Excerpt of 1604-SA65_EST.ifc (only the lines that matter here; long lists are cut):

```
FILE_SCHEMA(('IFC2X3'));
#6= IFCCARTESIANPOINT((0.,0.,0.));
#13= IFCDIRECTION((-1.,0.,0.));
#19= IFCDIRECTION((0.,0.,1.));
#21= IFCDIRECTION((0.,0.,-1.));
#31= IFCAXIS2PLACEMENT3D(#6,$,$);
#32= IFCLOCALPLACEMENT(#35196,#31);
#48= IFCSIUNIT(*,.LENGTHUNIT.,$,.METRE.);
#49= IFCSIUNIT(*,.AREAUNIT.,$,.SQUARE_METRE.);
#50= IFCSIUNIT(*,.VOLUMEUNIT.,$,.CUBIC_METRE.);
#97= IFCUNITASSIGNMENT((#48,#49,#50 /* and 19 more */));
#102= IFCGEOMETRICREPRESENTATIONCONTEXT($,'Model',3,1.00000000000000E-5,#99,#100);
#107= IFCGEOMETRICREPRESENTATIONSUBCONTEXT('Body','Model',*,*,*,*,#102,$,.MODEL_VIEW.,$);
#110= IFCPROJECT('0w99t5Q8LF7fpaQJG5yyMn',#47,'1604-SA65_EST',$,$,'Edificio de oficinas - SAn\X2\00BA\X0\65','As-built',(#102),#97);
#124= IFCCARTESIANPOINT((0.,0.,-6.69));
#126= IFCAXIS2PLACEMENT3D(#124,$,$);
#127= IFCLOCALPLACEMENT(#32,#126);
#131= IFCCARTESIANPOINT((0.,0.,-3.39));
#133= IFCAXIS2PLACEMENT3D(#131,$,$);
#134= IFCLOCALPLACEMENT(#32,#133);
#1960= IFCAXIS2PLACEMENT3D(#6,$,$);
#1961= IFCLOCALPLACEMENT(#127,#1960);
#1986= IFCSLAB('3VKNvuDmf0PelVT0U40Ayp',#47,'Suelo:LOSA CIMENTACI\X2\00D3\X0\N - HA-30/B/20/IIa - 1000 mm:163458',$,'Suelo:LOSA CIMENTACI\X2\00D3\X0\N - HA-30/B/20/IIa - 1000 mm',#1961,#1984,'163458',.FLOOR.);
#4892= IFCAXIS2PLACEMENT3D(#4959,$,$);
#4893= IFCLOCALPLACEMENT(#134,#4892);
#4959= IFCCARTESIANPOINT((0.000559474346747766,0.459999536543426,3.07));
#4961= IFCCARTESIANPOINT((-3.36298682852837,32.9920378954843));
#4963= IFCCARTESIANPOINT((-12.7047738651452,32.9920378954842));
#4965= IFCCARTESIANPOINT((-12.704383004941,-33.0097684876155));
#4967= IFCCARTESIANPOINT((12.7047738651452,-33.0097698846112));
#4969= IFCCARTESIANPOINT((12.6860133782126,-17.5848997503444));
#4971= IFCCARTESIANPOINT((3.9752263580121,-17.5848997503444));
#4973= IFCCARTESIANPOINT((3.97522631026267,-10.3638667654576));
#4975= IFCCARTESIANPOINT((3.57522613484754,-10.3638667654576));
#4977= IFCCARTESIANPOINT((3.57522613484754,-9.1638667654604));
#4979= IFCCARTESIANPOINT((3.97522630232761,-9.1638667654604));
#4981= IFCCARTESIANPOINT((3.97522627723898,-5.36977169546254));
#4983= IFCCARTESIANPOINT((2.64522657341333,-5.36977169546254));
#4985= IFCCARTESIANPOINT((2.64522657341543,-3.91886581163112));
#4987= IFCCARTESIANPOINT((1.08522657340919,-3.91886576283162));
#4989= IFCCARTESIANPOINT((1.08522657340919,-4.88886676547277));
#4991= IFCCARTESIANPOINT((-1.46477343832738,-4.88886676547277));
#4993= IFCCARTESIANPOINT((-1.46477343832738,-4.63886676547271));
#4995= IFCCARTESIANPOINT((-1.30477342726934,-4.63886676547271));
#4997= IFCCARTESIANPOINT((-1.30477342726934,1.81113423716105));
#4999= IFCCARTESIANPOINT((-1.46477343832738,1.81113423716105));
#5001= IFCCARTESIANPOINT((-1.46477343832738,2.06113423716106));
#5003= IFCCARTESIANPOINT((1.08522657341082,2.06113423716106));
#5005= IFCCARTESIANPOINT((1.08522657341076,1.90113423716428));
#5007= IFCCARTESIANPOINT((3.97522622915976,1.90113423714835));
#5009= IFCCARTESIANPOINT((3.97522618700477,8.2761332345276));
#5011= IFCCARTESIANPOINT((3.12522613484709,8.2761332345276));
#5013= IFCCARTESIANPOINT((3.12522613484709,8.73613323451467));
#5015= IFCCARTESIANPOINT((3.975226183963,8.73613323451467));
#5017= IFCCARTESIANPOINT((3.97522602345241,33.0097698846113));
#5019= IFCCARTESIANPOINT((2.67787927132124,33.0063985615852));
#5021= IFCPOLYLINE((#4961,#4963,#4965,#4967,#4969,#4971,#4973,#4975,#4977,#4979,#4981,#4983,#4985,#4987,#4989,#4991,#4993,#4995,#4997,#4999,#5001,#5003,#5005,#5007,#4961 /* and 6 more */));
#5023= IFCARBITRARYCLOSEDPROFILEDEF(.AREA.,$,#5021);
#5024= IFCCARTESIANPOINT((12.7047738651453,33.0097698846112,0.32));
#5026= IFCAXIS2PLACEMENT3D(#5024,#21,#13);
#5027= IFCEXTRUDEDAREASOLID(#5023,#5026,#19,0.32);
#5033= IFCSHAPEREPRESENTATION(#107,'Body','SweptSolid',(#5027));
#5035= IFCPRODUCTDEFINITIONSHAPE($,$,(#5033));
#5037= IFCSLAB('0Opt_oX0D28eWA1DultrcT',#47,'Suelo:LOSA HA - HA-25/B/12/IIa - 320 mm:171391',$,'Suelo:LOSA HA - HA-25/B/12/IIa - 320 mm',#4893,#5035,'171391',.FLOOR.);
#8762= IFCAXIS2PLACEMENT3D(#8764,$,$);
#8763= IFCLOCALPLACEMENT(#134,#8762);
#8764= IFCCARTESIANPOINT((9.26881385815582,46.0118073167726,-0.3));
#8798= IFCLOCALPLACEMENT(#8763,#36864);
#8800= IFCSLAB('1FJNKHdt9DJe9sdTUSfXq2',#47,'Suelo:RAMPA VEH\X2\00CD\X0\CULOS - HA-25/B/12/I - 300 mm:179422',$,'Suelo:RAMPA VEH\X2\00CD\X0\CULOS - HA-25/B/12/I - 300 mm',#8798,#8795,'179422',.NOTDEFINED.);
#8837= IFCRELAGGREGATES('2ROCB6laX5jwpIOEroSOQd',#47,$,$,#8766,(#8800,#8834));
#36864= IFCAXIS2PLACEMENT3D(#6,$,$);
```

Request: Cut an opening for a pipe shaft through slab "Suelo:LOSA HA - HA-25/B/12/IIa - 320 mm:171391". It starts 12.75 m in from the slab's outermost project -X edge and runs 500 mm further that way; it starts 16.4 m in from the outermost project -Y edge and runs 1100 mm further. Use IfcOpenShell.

```python
import numpy as np
import ifcopenshell
import ifcopenshell.api.feature
import ifcopenshell.api.geometry
import ifcopenshell.api.root
import ifcopenshell.geom
import ifcopenshell.util.placement
import ifcopenshell.util.representation
import ifcopenshell.util.shape
import ifcopenshell.util.unit

model = ifcopenshell.open("1604-SA65_EST.ifc")
unit_scale = ifcopenshell.util.unit.calculate_unit_scale(model)
settings = ifcopenshell.geom.settings()


def volume(element):
    """Net volume in cubic metres, openings subtracted."""
    shape = ifcopenshell.geom.create_shape(settings, element)
    return ifcopenshell.util.shape.get_volume(shape.geometry)


slab = model.by_id(5037)
before = volume(slab)

# Extent in the slab's own axes, in metres. The edges named are its -X and -Y sides.
slab_shape = ifcopenshell.geom.create_shape(settings, slab)
vertices = ifcopenshell.util.shape.get_vertices(slab_shape.geometry)
x_min, y_min, bottom = vertices.min(axis=0)
top = vertices[:, 2].max()

opening = ifcopenshell.api.root.create_entity(model, ifc_class="IfcOpeningElement", name="Pipe shaft opening")
context = ifcopenshell.util.representation.get_context(model, "Model", "Body", "MODEL_VIEW")
width, depth = 0.5, 1.1
outline = [(0.0, 0.0), (width, 0.0), (width, depth), (0.0, depth), (0.0, 0.0)]
# Overshoot both faces by 50 mm so the cut is clean.
shape = ifcopenshell.api.geometry.add_slab_representation(
    model, context=context, depth=top - bottom + 0.1, polyline=outline
)
ifcopenshell.api.geometry.assign_representation(model, product=opening, representation=shape)

matrix = ifcopenshell.util.placement.get_local_placement(slab.ObjectPlacement)
matrix[:, 3] = matrix @ np.append(np.array([x_min + 12.75, y_min + 16.4, bottom - 0.05]) / unit_scale, 1.0)
ifcopenshell.api.geometry.edit_object_placement(model, product=opening, matrix=matrix, is_si=False)
ifcopenshell.api.feature.add_feature(model, feature=opening, element=slab)

after = volume(slab)

print(f"slab volume {before:.3f} -> {after:.3f} m3")

model.write("1604-SA65_EST-out.ifc")
```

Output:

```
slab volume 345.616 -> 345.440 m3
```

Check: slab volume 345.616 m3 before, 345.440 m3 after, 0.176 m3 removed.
